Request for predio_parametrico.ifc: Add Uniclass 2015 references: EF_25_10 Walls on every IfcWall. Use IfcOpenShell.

First a look at what the model holds.

```python
import ifcopenshell

model = ifcopenshell.open("predio_parametrico.ifc")
print(model.schema)
print("classifications:", [c.Name for c in model.by_type("IfcClassification")])
for ifc_class in ("IfcDoor", "IfcRoof", "IfcStair", "IfcWall", "IfcWindow"):
    print(ifc_class, len(model.by_type(ifc_class)))
```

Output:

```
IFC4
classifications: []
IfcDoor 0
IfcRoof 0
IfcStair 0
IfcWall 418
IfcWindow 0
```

```python
import ifcopenshell
import ifcopenshell.api.classification

model = ifcopenshell.open("predio_parametrico.ifc")

system = ifcopenshell.api.classification.add_classification(model, classification="Uniclass 2015")

codes = {
    "IfcWall": ("EF_25_10", "Walls"),
}
for ifc_class, (code, name) in codes.items():
    products = model.by_type(ifc_class)
    ifcopenshell.api.classification.add_reference(
        model, products=products, classification=system, identification=code, name=name
    )
    print(code, len(products))

model.write("predio_parametrico_v2.ifc")
```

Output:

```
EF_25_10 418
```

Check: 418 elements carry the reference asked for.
